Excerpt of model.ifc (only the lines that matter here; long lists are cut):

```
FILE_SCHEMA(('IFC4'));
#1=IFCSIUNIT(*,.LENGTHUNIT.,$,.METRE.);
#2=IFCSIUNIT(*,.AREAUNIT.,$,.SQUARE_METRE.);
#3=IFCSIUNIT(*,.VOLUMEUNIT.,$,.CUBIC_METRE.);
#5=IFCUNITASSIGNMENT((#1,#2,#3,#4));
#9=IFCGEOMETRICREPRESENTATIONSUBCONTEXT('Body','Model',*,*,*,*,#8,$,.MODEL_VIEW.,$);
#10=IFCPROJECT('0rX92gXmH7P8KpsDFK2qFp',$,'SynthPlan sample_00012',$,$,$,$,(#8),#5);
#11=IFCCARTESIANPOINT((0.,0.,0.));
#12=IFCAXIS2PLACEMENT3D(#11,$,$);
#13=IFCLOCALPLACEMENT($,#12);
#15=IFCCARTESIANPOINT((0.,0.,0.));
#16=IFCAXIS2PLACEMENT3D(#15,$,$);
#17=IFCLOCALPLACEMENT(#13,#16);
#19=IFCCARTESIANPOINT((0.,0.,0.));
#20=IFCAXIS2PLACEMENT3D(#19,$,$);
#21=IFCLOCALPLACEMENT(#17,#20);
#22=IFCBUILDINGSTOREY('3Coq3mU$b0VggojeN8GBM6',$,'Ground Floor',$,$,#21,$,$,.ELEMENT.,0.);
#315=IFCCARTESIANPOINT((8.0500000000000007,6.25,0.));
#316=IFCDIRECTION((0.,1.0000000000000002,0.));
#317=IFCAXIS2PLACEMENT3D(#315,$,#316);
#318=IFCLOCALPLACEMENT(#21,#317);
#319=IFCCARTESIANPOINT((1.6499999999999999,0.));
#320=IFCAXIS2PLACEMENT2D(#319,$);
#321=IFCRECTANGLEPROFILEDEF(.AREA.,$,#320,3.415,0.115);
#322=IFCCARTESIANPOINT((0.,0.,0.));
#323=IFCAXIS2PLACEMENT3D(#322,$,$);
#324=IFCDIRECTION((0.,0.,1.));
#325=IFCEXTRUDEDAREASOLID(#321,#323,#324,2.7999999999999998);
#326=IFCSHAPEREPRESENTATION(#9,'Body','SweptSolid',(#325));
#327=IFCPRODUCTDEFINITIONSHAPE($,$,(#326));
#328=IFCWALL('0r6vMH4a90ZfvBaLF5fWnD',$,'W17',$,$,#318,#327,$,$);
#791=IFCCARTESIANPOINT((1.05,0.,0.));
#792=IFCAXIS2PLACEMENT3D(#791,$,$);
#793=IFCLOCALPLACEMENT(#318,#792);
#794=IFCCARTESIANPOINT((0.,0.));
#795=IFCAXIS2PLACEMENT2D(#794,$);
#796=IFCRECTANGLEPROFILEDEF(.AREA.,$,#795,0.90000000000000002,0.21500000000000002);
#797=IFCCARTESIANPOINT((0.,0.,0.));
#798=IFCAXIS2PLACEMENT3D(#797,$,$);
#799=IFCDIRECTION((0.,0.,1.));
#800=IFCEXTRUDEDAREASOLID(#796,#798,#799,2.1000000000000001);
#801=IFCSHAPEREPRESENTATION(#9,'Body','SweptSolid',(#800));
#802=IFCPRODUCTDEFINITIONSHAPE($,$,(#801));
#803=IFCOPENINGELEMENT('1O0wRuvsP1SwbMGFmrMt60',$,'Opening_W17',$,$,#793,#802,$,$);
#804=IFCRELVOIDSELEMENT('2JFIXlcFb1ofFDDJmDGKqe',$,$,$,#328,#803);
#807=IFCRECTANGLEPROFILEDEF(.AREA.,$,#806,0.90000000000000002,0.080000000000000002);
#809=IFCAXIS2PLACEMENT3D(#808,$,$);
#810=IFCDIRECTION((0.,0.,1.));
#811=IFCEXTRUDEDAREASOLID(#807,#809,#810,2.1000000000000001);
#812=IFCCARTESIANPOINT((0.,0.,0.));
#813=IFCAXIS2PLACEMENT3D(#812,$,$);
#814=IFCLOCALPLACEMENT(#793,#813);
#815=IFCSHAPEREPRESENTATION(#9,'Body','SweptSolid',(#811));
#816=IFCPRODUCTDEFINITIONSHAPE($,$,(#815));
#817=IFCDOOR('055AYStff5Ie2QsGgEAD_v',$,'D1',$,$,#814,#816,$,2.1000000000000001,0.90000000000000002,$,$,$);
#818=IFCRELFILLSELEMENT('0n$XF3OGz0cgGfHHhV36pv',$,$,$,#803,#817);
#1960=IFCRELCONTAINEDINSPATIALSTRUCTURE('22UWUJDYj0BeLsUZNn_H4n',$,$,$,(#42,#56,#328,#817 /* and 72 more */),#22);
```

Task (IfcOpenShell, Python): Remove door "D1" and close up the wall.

```python
import ifcopenshell
import ifcopenshell.api.feature
import ifcopenshell.api.root
import ifcopenshell.geom
import ifcopenshell.util.shape

model = ifcopenshell.open("model.ifc")
settings = ifcopenshell.geom.settings()


def volume(element):
    """Net volume in cubic metres, openings subtracted."""
    shape = ifcopenshell.geom.create_shape(settings, element)
    return ifcopenshell.util.shape.get_volume(shape.geometry)


door = model.by_guid("055AYStff5Ie2QsGgEAD_v")
opening = door.FillsVoids[0].RelatingOpeningElement
wall = opening.VoidsElements[0].RelatingBuildingElement
before = volume(wall)

ifcopenshell.api.root.remove_product(model, product=door)
ifcopenshell.api.feature.remove_feature(model, feature=opening)

after = volume(wall)

print(f"wall volume {before:.3f} -> {after:.3f} m3")

model.write("model_edited.ifc")
```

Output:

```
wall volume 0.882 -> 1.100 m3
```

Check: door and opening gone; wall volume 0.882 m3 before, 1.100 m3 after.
